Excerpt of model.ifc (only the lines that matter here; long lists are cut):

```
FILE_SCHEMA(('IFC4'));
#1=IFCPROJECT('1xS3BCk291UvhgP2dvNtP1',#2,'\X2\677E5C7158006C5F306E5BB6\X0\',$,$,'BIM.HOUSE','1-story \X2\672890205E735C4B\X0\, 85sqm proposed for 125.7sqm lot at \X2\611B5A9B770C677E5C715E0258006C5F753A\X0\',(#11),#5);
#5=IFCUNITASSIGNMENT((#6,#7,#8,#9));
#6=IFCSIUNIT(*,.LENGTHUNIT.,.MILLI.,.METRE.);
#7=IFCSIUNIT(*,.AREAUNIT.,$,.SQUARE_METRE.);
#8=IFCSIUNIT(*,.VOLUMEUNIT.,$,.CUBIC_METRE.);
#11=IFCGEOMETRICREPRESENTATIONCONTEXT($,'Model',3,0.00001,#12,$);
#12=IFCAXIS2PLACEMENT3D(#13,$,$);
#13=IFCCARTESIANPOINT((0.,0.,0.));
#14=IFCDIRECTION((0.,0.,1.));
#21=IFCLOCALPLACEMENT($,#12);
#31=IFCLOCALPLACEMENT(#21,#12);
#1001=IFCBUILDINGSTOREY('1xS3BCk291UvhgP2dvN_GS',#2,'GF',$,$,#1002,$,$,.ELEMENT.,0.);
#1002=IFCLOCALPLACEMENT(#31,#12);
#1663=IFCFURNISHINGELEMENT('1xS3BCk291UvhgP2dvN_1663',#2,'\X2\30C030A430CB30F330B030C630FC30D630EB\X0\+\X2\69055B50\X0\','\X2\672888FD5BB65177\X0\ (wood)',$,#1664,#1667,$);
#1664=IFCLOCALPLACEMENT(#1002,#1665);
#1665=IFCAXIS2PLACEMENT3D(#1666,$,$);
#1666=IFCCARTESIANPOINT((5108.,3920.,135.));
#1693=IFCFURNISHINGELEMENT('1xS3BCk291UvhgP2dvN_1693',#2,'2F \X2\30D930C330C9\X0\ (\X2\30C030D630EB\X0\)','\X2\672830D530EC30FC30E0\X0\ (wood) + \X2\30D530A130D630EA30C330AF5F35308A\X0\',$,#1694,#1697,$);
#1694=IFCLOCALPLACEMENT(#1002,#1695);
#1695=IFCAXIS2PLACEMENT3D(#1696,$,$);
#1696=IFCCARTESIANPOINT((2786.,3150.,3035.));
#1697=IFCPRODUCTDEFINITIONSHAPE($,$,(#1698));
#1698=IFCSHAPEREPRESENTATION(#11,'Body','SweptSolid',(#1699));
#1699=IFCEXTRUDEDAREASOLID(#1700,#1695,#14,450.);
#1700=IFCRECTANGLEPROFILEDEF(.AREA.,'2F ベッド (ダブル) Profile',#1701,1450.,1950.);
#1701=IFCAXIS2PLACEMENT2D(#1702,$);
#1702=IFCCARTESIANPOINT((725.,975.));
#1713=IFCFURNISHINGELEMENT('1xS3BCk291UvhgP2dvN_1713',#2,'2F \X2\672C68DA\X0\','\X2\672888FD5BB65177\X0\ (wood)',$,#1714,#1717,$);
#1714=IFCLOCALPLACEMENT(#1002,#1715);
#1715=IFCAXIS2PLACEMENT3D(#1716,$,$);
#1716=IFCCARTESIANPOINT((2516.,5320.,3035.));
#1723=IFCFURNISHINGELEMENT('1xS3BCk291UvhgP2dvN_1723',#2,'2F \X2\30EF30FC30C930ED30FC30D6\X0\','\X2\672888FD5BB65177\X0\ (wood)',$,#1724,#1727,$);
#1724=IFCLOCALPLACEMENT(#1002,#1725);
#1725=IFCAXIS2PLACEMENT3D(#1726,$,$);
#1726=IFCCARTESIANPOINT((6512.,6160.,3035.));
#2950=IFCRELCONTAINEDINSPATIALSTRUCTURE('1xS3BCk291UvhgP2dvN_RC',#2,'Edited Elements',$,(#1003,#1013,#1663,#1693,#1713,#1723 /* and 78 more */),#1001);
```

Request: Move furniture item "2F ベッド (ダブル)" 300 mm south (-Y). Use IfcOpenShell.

```python
import ifcopenshell
import ifcopenshell.api.geometry
import ifcopenshell.util.placement
import ifcopenshell.util.unit

model = ifcopenshell.open("model.ifc")
unit_scale = ifcopenshell.util.unit.calculate_unit_scale(model)

item = model.by_id(1693)
matrix = ifcopenshell.util.placement.get_local_placement(item.ObjectPlacement)
matrix[1, 3] -= 0.3 / unit_scale
ifcopenshell.api.geometry.edit_object_placement(model, product=item, matrix=matrix, is_si=False)

print(ifcopenshell.util.placement.get_local_placement(item.ObjectPlacement).round(3) + 0.0)

model.write("model_v2.ifc")
```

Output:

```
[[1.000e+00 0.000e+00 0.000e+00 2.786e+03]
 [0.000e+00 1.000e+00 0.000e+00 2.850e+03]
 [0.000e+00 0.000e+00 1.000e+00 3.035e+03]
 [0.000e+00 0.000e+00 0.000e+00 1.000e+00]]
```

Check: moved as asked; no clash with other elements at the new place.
